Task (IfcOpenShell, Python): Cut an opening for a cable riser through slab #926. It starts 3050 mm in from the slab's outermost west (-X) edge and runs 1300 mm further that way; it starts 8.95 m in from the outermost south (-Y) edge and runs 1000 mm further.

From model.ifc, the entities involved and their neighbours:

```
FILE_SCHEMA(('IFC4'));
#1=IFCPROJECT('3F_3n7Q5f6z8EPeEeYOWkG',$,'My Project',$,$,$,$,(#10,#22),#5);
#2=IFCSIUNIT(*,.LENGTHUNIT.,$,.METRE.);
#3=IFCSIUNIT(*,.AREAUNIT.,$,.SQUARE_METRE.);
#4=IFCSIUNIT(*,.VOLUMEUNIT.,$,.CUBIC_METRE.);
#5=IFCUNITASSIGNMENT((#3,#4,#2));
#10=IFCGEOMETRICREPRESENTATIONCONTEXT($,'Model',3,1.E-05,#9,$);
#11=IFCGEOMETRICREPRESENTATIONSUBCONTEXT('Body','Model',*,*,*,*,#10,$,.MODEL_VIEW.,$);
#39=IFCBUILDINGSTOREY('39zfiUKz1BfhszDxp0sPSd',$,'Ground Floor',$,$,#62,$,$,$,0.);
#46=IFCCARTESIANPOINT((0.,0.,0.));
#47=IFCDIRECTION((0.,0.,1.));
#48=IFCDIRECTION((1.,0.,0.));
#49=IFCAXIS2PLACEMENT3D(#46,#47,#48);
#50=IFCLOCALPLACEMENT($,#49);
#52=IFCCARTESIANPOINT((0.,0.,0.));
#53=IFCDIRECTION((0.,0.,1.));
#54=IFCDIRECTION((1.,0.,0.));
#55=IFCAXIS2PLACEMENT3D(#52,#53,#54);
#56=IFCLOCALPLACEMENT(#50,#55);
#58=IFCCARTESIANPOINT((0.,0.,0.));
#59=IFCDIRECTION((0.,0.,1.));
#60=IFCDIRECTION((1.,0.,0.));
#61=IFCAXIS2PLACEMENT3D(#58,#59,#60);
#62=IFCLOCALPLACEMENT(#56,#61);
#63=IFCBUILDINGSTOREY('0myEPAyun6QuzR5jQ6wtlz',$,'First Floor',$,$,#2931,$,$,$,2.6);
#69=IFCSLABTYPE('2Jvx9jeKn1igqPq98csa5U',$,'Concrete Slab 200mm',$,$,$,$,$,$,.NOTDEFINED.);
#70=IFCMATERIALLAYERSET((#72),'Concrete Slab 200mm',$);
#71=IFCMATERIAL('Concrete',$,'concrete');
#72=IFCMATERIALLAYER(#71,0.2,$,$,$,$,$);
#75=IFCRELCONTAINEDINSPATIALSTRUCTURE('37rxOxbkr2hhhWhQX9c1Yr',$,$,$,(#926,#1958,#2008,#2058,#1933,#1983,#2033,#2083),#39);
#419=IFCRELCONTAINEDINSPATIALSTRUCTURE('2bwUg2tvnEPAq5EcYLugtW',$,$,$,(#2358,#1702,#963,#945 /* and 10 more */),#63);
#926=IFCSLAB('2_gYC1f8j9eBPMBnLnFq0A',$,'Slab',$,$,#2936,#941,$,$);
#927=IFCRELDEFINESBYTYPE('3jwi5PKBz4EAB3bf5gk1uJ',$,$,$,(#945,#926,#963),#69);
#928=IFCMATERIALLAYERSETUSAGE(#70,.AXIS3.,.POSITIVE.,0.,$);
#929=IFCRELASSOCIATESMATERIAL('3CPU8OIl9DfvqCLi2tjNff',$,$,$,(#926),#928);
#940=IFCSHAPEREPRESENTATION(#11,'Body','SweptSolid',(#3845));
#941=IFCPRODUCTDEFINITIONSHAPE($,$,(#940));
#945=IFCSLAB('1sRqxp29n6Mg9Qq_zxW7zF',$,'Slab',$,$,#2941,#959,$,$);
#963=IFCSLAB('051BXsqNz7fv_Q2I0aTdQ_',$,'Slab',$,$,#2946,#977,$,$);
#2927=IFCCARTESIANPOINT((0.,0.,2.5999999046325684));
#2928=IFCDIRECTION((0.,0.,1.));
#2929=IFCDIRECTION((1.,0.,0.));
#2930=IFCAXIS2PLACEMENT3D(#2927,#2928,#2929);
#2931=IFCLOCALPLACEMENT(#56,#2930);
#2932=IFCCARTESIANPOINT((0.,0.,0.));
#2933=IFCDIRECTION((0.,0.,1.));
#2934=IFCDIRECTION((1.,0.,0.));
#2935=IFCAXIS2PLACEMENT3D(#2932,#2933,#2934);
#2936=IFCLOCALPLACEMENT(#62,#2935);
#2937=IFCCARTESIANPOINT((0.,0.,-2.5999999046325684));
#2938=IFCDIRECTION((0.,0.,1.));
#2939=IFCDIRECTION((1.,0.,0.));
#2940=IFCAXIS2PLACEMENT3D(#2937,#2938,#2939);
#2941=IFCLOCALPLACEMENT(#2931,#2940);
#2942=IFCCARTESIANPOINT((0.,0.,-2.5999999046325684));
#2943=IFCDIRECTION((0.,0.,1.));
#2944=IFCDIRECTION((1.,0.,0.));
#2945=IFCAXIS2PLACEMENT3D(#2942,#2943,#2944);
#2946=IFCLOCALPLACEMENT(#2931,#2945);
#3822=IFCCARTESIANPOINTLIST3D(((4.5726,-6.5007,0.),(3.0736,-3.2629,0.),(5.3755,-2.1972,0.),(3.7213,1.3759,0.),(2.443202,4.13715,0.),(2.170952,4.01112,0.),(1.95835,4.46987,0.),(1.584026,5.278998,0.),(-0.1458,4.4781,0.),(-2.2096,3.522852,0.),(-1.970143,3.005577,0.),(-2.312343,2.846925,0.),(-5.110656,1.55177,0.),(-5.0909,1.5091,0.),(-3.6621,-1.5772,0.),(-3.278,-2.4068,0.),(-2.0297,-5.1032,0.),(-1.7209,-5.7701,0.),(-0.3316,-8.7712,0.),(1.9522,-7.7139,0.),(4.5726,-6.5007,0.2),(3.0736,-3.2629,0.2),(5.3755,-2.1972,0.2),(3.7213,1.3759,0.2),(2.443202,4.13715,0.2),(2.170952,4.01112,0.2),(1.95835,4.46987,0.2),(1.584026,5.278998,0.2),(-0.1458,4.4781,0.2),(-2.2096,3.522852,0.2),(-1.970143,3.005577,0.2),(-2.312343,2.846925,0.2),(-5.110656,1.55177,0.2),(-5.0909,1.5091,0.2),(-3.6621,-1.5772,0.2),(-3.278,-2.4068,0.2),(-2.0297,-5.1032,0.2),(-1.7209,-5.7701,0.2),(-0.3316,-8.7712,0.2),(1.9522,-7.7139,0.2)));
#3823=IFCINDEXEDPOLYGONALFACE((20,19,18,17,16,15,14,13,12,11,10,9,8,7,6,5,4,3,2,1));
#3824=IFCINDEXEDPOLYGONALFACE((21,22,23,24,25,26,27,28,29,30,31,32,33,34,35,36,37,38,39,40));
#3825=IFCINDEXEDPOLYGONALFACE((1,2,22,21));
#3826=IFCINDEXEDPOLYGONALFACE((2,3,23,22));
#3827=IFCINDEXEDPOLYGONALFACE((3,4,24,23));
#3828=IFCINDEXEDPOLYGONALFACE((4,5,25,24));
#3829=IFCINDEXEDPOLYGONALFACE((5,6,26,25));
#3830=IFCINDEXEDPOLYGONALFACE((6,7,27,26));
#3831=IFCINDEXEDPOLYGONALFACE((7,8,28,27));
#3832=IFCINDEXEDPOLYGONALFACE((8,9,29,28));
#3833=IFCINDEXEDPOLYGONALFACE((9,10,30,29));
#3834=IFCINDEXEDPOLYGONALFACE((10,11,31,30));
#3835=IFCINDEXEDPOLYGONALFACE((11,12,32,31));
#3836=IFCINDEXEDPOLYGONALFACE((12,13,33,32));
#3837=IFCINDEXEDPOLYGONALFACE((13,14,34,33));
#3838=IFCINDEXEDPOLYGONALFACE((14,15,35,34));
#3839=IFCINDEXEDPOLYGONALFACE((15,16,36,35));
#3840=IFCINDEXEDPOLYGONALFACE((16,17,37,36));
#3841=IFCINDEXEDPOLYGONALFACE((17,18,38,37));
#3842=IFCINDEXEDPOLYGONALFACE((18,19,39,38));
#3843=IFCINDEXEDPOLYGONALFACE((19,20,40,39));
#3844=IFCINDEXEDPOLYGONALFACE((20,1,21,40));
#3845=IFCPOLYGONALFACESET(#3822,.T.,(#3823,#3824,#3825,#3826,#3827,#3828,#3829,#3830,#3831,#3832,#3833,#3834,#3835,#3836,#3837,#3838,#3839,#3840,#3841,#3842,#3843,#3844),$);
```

```python
import numpy as np
import ifcopenshell
import ifcopenshell.api.feature
import ifcopenshell.api.geometry
import ifcopenshell.api.root
import ifcopenshell.geom
import ifcopenshell.util.placement
import ifcopenshell.util.representation
import ifcopenshell.util.shape
import ifcopenshell.util.unit

model = ifcopenshell.open("model.ifc")
unit_scale = ifcopenshell.util.unit.calculate_unit_scale(model)
settings = ifcopenshell.geom.settings()


def volume(element):
    """Net volume in cubic metres, openings subtracted."""
    shape = ifcopenshell.geom.create_shape(settings, element)
    return ifcopenshell.util.shape.get_volume(shape.geometry)


slab = model.by_id(926)
before = volume(slab)

# Extent in the slab's own axes, in metres. The edges named are its -X and -Y sides.
slab_shape = ifcopenshell.geom.create_shape(settings, slab)
vertices = ifcopenshell.util.shape.get_vertices(slab_shape.geometry)
x_min, y_min, bottom = vertices.min(axis=0)
top = vertices[:, 2].max()

opening = ifcopenshell.api.root.create_entity(model, ifc_class="IfcOpeningElement", name="Cable riser opening", predefined_type="OPENING")
context = ifcopenshell.util.representation.get_context(model, "Model", "Body", "MODEL_VIEW")
width, depth = 1.3, 1
outline = [(0.0, 0.0), (width, 0.0), (width, depth), (0.0, depth), (0.0, 0.0)]
# Overshoot both faces by 50 mm so the cut is clean.
shape = ifcopenshell.api.geometry.add_slab_representation(
    model, context=context, depth=top - bottom + 0.1, polyline=outline
)
ifcopenshell.api.geometry.assign_representation(model, product=opening, representation=shape)

matrix = ifcopenshell.util.placement.get_local_placement(slab.ObjectPlacement)
matrix[:, 3] = matrix @ np.append(np.array([x_min + 3.05, y_min + 8.95, bottom - 0.05]) / unit_scale, 1.0)
ifcopenshell.api.geometry.edit_object_placement(model, product=opening, matrix=matrix, is_si=False)
ifcopenshell.api.feature.add_feature(model, feature=opening, element=slab)

after = volume(slab)

print(f"slab volume {before:.3f} -> {after:.3f} m3")

model.write("model_edited.ifc")
```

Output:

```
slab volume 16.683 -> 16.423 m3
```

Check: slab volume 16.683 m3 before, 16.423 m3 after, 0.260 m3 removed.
